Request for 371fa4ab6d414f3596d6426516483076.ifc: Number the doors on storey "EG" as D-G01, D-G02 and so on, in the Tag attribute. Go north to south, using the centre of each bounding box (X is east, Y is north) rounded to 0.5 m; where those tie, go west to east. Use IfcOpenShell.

First a look at what the model holds.

```python
import ifcopenshell
import ifcopenshell.util.element
import ifcopenshell.util.placement

model = ifcopenshell.open("371fa4ab6d414f3596d6426516483076.ifc")
print(model.schema)
storey = next(s for s in model.by_type("IfcBuildingStorey") if s.Name == "EG")
doors = [e for e in ifcopenshell.util.element.get_decomposition(storey) if e.is_a("IfcDoor")]
for e in sorted(doors, key=lambda e: e.id()):
    origin = ifcopenshell.util.placement.get_local_placement(e.ObjectPlacement)[:3, 3]
    print(e.id(), e.Tag, e.Name, origin.round(2) + 0.0, sep=" | ")
```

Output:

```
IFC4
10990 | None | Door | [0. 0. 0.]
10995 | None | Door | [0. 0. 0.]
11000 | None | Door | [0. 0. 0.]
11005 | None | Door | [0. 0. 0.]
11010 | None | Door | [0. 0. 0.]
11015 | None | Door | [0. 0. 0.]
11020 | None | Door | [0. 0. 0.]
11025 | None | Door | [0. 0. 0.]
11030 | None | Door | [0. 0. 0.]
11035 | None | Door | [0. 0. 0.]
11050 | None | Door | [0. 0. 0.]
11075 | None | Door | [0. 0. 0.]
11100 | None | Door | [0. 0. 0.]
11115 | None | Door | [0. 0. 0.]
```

```python
import ifcopenshell
import ifcopenshell.geom
import ifcopenshell.util.element
import ifcopenshell.util.shape

model = ifcopenshell.open("371fa4ab6d414f3596d6426516483076.ifc")
settings = ifcopenshell.geom.settings()
settings.set("use-world-coords", True)


def centre(element):
    shape = ifcopenshell.geom.create_shape(settings, element)
    return ifcopenshell.util.shape.get_bbox_centroid(shape.geometry)


storey = next(s for s in model.by_type("IfcBuildingStorey") if s.Name == "EG")
doors = [e for e in ifcopenshell.util.element.get_decomposition(storey) if e.is_a("IfcDoor")]

# Insertion points can sit at a corner or the storey origin, so sort by the geometry (in metres).
centres = {e: centre(e) for e in doors}
doors.sort(key=lambda e: (-round(centres[e][1] / 0.5), centres[e][0]))

for i, e in enumerate(doors, start=1):
    number = f"D-G{i:02d}"
    e.Tag = number
    print(e.id(), number)

model.write("371fa4ab6d414f3596d6426516483076_edited.ifc")
```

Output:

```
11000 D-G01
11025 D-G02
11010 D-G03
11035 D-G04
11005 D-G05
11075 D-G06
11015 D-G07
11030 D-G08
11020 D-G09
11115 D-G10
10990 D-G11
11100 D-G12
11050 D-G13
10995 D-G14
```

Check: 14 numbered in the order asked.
